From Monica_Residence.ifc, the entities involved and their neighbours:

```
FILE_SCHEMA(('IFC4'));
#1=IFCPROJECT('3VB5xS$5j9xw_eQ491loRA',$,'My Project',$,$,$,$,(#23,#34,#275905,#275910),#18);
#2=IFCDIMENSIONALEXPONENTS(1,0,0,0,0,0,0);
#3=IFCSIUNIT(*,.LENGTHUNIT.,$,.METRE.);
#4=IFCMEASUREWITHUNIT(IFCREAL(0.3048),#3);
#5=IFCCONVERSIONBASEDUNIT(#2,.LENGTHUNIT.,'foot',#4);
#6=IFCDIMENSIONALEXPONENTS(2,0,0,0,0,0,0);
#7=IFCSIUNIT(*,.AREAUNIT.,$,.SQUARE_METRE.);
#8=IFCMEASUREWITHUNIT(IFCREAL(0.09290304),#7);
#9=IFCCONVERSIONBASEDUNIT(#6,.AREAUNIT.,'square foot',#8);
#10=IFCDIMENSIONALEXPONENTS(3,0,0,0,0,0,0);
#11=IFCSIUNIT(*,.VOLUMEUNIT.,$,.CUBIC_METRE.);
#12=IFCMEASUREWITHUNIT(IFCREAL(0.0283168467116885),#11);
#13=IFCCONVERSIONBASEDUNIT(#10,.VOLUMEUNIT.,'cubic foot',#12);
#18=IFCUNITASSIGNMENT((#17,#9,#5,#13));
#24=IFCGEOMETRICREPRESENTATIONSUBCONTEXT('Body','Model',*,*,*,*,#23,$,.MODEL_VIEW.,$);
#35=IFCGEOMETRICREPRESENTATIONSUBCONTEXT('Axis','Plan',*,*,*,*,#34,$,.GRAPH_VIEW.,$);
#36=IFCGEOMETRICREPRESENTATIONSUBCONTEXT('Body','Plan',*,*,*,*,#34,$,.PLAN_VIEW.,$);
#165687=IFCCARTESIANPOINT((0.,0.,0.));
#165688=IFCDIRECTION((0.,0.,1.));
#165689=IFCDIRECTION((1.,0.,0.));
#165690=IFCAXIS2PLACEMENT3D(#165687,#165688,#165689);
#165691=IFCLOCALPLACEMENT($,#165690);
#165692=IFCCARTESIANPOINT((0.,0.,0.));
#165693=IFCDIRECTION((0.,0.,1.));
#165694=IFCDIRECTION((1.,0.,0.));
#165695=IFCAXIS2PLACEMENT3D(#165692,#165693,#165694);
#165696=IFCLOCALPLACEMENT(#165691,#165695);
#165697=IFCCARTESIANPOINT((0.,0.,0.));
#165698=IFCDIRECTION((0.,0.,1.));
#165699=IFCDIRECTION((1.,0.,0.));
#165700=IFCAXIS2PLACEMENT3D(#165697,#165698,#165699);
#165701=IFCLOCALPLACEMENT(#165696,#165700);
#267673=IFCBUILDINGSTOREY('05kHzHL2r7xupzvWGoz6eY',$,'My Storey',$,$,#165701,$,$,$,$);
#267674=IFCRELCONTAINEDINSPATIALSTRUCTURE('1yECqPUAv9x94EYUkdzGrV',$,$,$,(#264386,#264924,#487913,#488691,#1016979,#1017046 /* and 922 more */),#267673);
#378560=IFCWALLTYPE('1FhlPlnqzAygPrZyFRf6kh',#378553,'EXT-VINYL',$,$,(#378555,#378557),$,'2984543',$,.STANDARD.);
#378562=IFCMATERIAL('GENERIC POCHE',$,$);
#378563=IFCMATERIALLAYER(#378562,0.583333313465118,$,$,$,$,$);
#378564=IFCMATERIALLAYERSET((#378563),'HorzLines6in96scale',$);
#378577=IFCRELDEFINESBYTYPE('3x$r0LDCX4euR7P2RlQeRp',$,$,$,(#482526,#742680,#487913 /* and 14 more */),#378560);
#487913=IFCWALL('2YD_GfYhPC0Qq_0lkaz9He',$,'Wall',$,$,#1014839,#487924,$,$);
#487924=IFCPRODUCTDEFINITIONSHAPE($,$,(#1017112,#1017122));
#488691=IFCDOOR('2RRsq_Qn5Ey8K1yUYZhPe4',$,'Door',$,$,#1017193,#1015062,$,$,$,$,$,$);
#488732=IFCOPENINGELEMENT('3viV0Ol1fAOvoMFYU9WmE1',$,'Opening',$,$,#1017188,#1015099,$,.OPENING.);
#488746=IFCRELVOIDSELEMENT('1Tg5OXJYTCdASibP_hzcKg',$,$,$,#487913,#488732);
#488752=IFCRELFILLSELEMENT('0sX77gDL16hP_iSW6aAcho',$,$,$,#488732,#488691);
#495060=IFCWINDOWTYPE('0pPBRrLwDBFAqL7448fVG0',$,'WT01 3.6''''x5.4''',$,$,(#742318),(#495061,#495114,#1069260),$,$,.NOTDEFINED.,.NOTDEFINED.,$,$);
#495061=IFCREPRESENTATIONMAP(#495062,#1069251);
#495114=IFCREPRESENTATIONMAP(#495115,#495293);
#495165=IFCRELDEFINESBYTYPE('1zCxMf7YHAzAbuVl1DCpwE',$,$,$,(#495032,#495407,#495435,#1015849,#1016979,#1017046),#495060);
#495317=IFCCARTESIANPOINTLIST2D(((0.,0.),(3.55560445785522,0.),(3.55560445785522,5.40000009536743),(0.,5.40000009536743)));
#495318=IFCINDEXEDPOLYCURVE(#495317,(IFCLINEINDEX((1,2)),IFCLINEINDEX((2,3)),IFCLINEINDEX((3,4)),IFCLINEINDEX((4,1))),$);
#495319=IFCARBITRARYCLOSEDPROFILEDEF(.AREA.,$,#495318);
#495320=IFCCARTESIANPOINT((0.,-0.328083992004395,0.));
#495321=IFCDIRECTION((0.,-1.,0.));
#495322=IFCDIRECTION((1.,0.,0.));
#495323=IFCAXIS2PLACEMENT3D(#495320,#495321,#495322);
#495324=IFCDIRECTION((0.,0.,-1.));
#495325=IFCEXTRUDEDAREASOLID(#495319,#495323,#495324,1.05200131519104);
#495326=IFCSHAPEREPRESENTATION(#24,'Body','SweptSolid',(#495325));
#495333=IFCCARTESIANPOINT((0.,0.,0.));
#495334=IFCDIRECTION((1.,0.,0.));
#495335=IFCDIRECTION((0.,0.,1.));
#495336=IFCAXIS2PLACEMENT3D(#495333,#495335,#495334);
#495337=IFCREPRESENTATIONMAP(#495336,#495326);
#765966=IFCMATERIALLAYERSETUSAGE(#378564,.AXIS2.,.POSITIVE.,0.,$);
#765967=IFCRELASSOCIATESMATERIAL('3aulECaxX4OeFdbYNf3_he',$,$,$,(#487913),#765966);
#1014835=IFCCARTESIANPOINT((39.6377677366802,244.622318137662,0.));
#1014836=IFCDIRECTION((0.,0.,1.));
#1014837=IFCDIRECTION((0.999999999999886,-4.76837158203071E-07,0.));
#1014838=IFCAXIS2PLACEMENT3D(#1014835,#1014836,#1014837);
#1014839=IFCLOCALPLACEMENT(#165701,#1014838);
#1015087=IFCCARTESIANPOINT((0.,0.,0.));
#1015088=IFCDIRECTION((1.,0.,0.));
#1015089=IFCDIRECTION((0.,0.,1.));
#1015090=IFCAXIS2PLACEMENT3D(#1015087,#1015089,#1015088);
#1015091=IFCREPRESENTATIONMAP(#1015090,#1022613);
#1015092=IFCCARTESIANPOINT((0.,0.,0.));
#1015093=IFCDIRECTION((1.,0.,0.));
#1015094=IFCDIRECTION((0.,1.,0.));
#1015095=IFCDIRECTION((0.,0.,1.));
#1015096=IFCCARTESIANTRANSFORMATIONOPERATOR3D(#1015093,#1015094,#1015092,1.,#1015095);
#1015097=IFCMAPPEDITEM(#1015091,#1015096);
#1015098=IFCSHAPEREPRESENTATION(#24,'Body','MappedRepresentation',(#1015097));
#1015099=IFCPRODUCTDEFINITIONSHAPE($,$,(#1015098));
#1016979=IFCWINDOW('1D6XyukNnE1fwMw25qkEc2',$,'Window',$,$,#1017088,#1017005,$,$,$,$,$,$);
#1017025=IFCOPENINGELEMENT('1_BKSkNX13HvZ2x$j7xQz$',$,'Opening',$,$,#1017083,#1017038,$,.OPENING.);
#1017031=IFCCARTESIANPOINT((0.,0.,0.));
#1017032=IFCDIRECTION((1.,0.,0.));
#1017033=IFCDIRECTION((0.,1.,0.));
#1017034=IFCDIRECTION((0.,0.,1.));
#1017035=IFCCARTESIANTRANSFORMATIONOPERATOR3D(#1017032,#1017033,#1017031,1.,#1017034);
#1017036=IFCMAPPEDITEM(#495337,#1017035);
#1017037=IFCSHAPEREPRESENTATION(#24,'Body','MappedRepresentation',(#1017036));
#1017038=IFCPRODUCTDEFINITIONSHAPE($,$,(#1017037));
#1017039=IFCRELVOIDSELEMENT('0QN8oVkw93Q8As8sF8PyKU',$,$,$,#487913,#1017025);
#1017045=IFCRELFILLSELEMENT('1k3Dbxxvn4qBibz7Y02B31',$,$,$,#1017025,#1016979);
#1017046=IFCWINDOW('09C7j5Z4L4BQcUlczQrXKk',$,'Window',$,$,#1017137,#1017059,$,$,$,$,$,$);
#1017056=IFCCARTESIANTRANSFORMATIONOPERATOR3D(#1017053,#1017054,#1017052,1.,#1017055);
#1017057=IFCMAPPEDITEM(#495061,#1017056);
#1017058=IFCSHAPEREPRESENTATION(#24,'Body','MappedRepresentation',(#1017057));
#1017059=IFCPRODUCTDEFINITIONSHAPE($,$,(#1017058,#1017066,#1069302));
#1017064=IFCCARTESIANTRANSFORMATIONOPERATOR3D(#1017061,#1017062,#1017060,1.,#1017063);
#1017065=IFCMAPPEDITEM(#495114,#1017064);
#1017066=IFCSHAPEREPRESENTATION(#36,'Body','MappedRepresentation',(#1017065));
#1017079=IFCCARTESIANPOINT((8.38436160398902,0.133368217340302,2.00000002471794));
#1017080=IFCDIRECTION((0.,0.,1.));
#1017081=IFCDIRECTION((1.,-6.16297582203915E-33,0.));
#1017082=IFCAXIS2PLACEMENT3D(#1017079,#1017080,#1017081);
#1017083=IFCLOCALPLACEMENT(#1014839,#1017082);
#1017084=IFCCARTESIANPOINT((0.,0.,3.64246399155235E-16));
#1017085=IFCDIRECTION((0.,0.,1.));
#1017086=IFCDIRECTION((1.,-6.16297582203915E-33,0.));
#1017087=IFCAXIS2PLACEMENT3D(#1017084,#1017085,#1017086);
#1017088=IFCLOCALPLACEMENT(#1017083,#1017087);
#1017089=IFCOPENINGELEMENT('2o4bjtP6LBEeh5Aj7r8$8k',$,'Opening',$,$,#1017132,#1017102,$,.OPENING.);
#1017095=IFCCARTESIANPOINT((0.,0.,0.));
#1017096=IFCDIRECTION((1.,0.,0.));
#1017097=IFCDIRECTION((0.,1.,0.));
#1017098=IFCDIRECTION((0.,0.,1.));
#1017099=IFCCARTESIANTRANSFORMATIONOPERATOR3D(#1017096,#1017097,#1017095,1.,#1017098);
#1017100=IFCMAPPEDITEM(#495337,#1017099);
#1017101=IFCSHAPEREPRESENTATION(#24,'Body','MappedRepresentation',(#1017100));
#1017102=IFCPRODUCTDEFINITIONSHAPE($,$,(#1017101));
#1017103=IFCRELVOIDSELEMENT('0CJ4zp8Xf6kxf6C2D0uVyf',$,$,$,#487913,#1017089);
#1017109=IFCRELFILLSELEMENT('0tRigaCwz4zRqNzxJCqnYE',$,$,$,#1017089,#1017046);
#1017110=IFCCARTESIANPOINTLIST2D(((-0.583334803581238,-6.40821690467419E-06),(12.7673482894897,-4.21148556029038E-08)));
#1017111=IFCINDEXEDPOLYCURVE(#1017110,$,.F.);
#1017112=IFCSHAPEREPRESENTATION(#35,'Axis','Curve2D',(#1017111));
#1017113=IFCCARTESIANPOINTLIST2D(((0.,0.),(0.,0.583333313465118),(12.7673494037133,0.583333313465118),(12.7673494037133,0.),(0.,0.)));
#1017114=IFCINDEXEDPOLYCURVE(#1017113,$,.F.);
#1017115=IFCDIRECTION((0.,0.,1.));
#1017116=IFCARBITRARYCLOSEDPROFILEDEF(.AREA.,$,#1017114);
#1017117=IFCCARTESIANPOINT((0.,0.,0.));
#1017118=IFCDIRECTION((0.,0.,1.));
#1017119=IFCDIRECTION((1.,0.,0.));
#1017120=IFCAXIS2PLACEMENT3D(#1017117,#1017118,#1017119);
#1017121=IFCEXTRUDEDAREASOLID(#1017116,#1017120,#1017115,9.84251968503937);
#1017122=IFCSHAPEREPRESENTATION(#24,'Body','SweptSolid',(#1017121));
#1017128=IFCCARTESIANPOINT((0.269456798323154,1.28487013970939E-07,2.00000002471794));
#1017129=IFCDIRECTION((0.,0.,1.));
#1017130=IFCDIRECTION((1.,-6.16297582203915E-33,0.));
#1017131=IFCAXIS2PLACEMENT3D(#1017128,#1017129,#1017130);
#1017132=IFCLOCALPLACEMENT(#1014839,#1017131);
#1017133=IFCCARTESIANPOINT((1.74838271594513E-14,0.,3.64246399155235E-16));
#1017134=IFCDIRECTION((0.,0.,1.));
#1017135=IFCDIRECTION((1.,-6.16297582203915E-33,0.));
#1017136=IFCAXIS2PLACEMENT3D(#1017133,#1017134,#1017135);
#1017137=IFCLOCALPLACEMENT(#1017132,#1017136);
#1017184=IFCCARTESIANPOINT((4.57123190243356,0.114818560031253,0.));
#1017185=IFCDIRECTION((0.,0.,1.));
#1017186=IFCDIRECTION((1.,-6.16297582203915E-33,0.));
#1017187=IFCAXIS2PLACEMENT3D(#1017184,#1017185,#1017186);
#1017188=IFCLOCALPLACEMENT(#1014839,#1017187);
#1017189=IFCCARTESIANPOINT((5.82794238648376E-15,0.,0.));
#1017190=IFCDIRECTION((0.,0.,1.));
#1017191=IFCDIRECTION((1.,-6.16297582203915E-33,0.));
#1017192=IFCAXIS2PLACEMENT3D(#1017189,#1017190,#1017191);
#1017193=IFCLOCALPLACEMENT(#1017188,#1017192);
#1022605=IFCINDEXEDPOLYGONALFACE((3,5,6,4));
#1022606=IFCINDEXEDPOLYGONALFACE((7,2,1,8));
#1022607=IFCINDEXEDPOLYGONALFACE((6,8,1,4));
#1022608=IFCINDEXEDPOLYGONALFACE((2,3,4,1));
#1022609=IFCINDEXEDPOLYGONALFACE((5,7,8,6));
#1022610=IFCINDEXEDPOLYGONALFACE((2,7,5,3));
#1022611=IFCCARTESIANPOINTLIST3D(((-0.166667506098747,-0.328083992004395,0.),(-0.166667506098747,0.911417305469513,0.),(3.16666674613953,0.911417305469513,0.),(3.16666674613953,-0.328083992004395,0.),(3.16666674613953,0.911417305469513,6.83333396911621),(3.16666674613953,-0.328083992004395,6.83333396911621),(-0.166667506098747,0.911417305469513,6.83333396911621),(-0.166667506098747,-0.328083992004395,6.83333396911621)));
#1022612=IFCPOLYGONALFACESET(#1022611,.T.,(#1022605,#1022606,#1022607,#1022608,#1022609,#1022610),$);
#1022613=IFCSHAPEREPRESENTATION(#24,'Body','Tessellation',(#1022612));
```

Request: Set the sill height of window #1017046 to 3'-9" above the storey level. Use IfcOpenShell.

```python
import numpy as np
import ifcopenshell
import ifcopenshell.api.geometry
import ifcopenshell.geom
import ifcopenshell.util.element
import ifcopenshell.util.placement
import ifcopenshell.util.shape
import ifcopenshell.util.unit

model = ifcopenshell.open("Monica_Residence.ifc")
unit_scale = ifcopenshell.util.unit.calculate_unit_scale(model)

window = model.by_id(1017046)
opening = window.FillsVoids[0].RelatingOpeningElement
storey = ifcopenshell.util.element.get_container(window, ifc_class="IfcBuildingStorey")
level = ifcopenshell.util.placement.get_local_placement(storey.ObjectPlacement)[2, 3]

# The opening's origin need not be at the sill, so measure its lowest point.
shape = ifcopenshell.geom.create_shape(ifcopenshell.geom.settings(), opening)
bottom = ifcopenshell.util.shape.get_shape_bottom_elevation(shape, shape.geometry) / unit_scale
dz = level + 45 * 0.0254 / unit_scale - bottom

shift = np.array([0.0, 0.0, dz])
# The window is placed relative to its opening, so it follows when the opening moves.
matrix = ifcopenshell.util.placement.get_local_placement(opening.ObjectPlacement)
matrix[:3, 3] += shift
ifcopenshell.api.geometry.edit_object_placement(
    model, product=opening, matrix=matrix, is_si=False, should_transform_children=True
)

print(f"moved by {dz * unit_scale:+.3f} m")

model.write("Monica_Residence_rev.ifc")
```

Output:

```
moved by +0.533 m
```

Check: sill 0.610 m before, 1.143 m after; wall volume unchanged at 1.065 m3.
